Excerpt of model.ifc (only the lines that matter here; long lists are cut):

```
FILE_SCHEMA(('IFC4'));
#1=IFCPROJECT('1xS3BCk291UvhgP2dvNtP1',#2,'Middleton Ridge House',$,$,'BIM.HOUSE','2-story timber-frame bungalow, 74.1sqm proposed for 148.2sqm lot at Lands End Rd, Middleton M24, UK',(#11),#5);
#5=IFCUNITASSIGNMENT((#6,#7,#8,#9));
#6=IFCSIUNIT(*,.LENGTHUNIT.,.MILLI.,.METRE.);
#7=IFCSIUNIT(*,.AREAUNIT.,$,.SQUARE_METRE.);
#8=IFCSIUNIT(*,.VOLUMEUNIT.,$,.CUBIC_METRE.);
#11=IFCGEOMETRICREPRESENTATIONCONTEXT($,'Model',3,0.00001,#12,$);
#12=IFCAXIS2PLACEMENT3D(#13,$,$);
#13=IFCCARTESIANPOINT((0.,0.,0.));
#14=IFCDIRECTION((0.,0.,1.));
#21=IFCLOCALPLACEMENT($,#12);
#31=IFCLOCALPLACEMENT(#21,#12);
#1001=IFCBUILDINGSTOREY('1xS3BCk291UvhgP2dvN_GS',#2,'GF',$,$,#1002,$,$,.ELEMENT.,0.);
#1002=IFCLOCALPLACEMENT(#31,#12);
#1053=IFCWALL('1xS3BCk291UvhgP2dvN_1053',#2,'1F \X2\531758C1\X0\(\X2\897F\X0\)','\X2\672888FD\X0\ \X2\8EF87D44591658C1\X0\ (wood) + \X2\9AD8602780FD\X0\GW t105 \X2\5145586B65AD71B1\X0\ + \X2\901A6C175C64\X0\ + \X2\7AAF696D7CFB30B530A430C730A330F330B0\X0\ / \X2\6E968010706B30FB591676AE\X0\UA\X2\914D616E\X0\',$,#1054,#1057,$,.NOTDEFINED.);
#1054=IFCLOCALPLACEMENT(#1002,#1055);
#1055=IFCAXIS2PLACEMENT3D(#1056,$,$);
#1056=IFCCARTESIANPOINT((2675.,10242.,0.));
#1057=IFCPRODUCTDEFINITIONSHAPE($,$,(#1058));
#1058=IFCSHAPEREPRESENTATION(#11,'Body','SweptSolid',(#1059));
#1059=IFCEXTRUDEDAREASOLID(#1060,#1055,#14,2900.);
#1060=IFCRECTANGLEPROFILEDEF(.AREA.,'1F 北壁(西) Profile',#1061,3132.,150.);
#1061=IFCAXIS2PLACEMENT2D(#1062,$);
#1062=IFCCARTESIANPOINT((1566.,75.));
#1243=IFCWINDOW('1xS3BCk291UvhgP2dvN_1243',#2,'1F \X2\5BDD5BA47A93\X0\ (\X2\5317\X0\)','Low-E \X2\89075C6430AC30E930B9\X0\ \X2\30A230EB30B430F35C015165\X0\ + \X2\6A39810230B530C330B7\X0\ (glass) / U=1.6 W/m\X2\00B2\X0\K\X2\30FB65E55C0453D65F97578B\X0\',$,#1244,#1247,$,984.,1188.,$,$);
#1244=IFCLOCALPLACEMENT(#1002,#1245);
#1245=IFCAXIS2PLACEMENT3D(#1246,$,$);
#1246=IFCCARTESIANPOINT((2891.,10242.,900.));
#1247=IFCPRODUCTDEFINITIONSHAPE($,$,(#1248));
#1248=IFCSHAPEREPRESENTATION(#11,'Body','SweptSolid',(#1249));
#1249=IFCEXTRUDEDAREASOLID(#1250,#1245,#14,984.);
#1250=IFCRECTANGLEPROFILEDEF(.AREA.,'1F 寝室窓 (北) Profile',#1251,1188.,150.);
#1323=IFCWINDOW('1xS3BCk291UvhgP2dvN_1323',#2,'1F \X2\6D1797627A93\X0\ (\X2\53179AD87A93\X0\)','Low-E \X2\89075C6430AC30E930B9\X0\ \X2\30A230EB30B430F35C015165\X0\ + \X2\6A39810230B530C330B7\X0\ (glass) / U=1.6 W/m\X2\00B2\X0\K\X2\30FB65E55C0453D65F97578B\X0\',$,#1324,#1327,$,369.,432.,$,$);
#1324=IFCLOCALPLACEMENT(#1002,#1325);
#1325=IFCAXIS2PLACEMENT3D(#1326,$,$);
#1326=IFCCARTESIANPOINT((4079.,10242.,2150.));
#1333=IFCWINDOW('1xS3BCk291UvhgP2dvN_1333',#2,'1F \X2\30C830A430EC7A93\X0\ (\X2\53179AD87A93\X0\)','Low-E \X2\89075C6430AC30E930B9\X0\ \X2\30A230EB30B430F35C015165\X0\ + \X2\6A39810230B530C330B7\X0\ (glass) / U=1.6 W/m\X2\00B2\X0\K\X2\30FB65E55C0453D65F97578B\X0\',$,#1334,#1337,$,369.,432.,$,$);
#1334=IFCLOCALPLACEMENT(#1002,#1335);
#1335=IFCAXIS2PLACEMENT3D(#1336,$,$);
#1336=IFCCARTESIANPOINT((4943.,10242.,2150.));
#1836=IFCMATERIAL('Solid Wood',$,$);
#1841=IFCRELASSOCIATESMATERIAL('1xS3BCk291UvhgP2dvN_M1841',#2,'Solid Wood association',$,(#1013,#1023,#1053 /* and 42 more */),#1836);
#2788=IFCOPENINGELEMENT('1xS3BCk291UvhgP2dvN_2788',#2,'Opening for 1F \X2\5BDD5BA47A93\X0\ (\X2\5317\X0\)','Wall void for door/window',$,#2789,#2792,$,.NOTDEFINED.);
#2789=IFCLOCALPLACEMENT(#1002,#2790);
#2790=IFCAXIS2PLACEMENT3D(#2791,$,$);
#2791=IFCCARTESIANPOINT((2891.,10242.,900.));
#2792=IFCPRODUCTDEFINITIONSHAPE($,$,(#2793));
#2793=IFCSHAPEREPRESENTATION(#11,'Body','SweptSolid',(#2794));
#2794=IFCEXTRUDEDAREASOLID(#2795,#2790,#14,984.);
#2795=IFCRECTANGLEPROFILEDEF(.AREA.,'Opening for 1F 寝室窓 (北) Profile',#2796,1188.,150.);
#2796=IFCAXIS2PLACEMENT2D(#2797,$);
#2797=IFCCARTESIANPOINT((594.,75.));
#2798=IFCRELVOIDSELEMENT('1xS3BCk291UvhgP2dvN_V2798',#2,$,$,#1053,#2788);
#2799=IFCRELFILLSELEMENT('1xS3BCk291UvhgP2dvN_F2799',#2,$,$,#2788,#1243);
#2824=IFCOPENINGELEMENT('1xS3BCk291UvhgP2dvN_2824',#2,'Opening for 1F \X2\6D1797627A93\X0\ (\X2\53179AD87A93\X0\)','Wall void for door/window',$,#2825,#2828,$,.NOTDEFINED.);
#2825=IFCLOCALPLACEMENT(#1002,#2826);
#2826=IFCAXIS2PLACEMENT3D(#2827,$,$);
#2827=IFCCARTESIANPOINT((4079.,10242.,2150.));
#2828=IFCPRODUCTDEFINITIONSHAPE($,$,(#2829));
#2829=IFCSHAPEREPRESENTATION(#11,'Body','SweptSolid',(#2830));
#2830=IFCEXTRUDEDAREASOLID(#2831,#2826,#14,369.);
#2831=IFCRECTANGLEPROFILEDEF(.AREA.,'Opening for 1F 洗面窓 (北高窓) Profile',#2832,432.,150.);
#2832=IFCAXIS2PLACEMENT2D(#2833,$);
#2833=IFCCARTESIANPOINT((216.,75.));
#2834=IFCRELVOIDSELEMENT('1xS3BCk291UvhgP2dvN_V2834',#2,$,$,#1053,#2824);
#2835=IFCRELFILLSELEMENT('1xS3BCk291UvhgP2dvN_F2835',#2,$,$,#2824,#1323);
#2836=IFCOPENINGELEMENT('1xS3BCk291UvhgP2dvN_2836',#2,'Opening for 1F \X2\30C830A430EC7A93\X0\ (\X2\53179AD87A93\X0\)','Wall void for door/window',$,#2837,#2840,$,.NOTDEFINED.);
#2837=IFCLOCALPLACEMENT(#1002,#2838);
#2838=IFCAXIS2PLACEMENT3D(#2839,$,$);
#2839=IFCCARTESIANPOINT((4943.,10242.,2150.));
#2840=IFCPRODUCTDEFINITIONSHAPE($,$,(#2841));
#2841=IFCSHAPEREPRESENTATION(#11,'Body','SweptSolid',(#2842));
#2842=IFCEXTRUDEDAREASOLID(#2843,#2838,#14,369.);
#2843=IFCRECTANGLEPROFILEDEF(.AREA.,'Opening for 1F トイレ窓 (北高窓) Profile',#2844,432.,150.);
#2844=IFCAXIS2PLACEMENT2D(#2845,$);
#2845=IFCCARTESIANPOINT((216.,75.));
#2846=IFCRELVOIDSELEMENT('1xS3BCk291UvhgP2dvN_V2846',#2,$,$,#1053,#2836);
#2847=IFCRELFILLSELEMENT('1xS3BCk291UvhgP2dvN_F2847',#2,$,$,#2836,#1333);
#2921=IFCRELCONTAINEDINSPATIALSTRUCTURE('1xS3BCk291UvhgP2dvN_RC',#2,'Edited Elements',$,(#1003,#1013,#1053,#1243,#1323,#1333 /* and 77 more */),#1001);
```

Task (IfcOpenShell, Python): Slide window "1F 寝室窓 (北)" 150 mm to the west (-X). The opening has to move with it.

```python
import ifcopenshell
import ifcopenshell.api.geometry
import ifcopenshell.util.placement
import ifcopenshell.util.unit

model = ifcopenshell.open("model.ifc")
unit_scale = ifcopenshell.util.unit.calculate_unit_scale(model)

window = model.by_guid("1xS3BCk291UvhgP2dvN_1243")
opening = window.FillsVoids[0].RelatingOpeningElement
wall = opening.VoidsElements[0].RelatingBuildingElement

wall_matrix = ifcopenshell.util.placement.get_local_placement(wall.ObjectPlacement)
shift = wall_matrix[:3, 0] * -0.15 / unit_scale
before = ifcopenshell.util.placement.get_local_placement(window.ObjectPlacement)[:3, 3].copy()

# The window is not placed relative to its opening, so move both.
for product in (opening, window):
    matrix = ifcopenshell.util.placement.get_local_placement(product.ObjectPlacement)
    matrix[:3, 3] += shift
    ifcopenshell.api.geometry.edit_object_placement(model, product=product, matrix=matrix, is_si=False)

after = ifcopenshell.util.placement.get_local_placement(window.ObjectPlacement)[:3, 3]
print("window moved by", (after - before).round(3) + 0.0)

model.write("model_v2.ifc")
```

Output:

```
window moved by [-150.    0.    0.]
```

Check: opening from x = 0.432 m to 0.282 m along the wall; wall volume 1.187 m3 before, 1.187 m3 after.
